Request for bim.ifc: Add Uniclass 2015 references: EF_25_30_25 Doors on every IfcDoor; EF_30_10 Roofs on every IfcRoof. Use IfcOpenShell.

First a look at what the model holds.

```python
import ifcopenshell

model = ifcopenshell.open("bim.ifc")
print(model.schema)
print("classifications:", [c.Name for c in model.by_type("IfcClassification")])
for ifc_class in ("IfcDoor", "IfcRoof", "IfcStair", "IfcWall", "IfcWindow"):
    print(ifc_class, len(model.by_type(ifc_class)))
```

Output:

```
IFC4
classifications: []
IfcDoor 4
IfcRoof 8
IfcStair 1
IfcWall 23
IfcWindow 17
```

```python
import ifcopenshell
import ifcopenshell.api.classification

model = ifcopenshell.open("bim.ifc")

system = ifcopenshell.api.classification.add_classification(model, classification="Uniclass 2015")

codes = {
    "IfcDoor": ("EF_25_30_25", "Doors"),
    "IfcRoof": ("EF_30_10", "Roofs"),
}
for ifc_class, (code, name) in codes.items():
    products = model.by_type(ifc_class)
    ifcopenshell.api.classification.add_reference(
        model, products=products, classification=system, identification=code, name=name
    )
    print(code, len(products))

model.write("bim_edited.ifc")
```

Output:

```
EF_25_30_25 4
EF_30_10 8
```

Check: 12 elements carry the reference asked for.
